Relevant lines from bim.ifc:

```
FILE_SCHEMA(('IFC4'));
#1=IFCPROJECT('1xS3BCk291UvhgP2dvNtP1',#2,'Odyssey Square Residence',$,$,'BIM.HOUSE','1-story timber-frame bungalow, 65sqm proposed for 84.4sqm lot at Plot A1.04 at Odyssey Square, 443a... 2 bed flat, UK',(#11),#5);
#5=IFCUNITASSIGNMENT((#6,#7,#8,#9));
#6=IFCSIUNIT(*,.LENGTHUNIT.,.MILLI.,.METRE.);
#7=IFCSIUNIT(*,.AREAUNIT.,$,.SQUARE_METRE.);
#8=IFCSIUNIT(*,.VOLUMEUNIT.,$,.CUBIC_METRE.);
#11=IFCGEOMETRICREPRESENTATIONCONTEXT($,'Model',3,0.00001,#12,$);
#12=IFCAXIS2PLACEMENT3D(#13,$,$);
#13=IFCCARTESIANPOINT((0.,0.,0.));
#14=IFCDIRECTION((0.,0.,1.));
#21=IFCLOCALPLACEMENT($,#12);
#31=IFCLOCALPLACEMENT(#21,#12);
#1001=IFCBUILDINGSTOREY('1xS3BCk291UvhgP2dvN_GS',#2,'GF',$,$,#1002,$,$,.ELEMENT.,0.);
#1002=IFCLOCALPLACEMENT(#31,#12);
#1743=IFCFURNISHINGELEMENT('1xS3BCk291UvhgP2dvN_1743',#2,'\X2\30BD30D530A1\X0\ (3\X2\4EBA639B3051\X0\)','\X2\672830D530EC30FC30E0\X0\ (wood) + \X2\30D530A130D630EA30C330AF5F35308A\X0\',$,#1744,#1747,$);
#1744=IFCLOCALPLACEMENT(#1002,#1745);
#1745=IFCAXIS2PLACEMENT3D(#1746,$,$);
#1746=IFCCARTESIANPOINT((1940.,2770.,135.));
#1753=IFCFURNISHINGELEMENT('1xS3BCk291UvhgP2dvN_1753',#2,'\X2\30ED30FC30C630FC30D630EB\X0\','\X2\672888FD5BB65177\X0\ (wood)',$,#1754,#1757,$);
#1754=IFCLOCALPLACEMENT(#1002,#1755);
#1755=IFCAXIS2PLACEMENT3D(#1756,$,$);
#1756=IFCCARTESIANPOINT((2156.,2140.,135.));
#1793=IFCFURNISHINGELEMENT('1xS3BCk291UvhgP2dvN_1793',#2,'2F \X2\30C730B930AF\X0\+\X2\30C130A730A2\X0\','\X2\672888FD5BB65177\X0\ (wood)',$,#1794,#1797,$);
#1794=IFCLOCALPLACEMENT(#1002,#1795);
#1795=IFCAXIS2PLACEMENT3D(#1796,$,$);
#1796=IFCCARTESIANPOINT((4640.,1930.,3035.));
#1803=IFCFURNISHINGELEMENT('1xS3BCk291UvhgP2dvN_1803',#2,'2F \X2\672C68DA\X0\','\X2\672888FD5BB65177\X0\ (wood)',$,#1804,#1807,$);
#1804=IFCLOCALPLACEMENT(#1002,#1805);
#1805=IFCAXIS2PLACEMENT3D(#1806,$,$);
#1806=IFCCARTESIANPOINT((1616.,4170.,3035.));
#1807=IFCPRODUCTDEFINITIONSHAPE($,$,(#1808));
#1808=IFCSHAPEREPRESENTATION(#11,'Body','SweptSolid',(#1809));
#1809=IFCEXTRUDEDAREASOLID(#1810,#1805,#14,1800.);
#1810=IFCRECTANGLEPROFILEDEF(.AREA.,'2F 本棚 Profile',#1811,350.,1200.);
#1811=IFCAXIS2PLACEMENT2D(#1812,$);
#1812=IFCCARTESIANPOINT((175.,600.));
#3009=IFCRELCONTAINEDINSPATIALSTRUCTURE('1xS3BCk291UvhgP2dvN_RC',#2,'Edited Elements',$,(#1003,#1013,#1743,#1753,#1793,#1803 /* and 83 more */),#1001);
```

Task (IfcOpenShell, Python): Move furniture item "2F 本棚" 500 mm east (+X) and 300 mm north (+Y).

```python
import ifcopenshell
import ifcopenshell.api.geometry
import ifcopenshell.util.placement
import ifcopenshell.util.unit

model = ifcopenshell.open("bim.ifc")
unit_scale = ifcopenshell.util.unit.calculate_unit_scale(model)

item = model.by_guid("1xS3BCk291UvhgP2dvN_1803")
matrix = ifcopenshell.util.placement.get_local_placement(item.ObjectPlacement)
matrix[0, 3] += 0.5 / unit_scale
matrix[1, 3] += 0.3 / unit_scale
ifcopenshell.api.geometry.edit_object_placement(model, product=item, matrix=matrix, is_si=False)

print(ifcopenshell.util.placement.get_local_placement(item.ObjectPlacement).round(3) + 0.0)

model.write("bim_rev.ifc")
```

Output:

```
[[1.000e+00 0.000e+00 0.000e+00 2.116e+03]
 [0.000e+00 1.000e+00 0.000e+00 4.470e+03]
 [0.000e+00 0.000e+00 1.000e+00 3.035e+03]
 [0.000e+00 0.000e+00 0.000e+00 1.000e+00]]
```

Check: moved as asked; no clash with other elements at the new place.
